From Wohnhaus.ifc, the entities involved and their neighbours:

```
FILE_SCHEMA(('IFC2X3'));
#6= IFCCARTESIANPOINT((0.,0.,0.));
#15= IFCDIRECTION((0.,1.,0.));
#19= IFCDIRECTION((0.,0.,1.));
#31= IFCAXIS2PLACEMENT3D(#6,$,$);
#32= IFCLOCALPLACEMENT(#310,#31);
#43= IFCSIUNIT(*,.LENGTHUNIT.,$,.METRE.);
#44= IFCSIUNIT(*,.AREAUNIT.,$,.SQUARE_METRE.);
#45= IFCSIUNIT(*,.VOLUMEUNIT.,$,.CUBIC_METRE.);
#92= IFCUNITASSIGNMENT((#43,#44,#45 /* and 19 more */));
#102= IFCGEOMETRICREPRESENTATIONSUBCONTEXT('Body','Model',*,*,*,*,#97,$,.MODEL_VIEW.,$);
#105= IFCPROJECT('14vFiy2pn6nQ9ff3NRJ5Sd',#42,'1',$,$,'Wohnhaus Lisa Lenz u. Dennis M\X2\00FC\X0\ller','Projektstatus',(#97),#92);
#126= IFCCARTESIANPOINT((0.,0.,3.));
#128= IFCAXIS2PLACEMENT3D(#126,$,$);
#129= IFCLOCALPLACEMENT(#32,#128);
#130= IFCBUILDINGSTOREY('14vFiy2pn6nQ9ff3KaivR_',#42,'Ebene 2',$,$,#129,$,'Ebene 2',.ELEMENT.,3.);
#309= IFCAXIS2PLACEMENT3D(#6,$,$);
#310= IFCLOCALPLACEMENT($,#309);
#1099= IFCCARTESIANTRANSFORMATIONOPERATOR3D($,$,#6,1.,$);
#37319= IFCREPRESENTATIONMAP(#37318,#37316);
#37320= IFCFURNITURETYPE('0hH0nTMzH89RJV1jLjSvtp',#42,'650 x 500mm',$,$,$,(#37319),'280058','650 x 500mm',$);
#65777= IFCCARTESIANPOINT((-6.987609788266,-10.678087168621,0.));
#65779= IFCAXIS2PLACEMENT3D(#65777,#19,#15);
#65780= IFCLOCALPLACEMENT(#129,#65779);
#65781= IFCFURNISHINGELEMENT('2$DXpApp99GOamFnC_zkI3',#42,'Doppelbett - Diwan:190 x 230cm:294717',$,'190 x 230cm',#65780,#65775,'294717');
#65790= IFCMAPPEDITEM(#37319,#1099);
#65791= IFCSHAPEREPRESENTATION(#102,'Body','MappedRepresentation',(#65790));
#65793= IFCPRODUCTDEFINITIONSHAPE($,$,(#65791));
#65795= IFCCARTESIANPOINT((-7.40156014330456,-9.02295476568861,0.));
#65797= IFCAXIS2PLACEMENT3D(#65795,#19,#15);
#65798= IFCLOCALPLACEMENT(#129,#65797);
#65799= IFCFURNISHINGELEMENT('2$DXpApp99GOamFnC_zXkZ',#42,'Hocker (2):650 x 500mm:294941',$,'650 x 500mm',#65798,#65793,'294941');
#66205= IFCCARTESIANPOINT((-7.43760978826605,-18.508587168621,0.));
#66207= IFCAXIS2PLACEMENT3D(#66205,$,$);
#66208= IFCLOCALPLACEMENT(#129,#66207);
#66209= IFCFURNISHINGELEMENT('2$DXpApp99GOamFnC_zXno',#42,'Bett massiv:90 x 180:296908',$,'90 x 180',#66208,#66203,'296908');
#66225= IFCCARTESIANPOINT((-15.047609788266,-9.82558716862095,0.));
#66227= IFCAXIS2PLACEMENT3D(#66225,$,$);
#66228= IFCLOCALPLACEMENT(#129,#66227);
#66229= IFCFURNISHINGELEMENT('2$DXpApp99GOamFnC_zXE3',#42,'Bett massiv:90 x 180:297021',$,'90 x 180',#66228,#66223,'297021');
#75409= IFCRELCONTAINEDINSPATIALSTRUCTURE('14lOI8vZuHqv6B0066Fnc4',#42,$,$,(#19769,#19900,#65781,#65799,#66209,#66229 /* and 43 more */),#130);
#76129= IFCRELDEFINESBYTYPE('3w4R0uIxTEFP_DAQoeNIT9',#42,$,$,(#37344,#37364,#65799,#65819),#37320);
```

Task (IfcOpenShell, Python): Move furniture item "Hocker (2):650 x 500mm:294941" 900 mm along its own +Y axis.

```python
import ifcopenshell
import ifcopenshell.api.geometry
import ifcopenshell.util.placement
import ifcopenshell.util.unit

model = ifcopenshell.open("Wohnhaus.ifc")
unit_scale = ifcopenshell.util.unit.calculate_unit_scale(model)

item = model.by_id(65799)
matrix = ifcopenshell.util.placement.get_local_placement(item.ObjectPlacement)
matrix[:3, 3] += matrix[:3, 1] * 0.9 / unit_scale
ifcopenshell.api.geometry.edit_object_placement(model, product=item, matrix=matrix, is_si=False)

print(ifcopenshell.util.placement.get_local_placement(item.ObjectPlacement).round(3) + 0.0)

model.write("Wohnhaus_updated.ifc")
```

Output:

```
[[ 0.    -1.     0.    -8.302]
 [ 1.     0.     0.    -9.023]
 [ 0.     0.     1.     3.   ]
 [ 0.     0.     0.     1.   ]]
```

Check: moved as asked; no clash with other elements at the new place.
